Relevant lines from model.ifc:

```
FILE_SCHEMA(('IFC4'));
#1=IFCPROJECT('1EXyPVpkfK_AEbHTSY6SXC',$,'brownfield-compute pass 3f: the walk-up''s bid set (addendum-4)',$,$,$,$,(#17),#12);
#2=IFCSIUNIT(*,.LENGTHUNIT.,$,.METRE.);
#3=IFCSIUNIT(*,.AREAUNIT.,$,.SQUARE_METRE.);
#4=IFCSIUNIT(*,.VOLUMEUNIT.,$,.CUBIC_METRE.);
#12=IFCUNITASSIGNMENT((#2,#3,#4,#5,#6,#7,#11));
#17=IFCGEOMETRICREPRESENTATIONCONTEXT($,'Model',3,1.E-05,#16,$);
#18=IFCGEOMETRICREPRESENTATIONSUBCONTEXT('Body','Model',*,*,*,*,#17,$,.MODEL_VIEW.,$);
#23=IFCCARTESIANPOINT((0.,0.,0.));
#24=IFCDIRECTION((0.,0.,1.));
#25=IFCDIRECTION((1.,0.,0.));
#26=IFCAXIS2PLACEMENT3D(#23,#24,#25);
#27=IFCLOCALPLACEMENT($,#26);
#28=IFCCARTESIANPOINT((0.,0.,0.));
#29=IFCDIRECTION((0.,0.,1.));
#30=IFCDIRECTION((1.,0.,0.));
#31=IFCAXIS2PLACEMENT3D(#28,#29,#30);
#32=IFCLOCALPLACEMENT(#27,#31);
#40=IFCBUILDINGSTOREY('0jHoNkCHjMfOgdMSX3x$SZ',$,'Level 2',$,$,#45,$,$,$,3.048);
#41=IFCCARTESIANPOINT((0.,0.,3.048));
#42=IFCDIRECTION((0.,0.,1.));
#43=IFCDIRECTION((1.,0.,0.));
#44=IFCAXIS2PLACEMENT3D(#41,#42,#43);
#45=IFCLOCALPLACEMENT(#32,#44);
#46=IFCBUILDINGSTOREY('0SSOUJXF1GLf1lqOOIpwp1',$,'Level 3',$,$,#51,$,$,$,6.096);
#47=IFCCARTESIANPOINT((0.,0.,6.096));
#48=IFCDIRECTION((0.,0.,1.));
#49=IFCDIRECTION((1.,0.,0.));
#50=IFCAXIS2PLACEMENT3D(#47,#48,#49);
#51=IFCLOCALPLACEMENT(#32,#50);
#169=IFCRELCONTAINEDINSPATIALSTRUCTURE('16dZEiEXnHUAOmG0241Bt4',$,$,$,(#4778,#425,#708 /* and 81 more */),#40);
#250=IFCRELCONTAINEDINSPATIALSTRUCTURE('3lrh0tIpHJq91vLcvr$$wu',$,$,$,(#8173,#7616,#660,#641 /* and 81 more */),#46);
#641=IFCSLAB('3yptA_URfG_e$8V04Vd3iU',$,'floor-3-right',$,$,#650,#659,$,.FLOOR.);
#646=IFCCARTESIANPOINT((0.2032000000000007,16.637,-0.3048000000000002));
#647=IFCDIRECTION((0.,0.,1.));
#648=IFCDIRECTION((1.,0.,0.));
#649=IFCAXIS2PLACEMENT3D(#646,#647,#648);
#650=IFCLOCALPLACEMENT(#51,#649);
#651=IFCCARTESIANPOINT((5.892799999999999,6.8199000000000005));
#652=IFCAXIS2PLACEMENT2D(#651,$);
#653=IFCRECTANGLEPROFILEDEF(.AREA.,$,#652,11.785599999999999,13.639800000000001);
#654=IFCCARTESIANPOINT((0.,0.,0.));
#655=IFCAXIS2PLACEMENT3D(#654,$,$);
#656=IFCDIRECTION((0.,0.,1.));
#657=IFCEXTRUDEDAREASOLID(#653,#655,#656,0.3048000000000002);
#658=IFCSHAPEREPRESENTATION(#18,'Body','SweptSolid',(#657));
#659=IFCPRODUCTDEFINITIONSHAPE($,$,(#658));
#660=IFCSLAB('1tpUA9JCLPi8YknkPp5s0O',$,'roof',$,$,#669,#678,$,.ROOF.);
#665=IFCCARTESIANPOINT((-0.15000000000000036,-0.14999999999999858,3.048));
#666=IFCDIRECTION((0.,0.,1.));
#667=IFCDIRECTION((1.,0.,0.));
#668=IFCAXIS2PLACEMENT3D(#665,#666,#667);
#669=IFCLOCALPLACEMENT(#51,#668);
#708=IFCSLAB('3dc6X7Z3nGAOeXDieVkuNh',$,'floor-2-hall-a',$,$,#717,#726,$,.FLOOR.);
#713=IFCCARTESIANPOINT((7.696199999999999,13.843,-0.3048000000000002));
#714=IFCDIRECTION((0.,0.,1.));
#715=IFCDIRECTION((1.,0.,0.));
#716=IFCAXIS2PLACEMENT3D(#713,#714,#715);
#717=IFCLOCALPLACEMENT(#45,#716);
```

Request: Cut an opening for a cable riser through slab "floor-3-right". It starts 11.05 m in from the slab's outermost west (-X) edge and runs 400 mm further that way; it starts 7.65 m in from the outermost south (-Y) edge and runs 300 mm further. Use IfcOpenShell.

```python
import numpy as np
import ifcopenshell
import ifcopenshell.api.feature
import ifcopenshell.api.geometry
import ifcopenshell.api.root
import ifcopenshell.geom
import ifcopenshell.util.placement
import ifcopenshell.util.representation
import ifcopenshell.util.shape
import ifcopenshell.util.unit

model = ifcopenshell.open("model.ifc")
unit_scale = ifcopenshell.util.unit.calculate_unit_scale(model)
settings = ifcopenshell.geom.settings()


def volume(element):
    """Net volume in cubic metres, openings subtracted."""
    shape = ifcopenshell.geom.create_shape(settings, element)
    return ifcopenshell.util.shape.get_volume(shape.geometry)


slab = model.by_guid("3yptA_URfG_e$8V04Vd3iU")
before = volume(slab)

# Extent in the slab's own axes, in metres. The edges named are its -X and -Y sides.
slab_shape = ifcopenshell.geom.create_shape(settings, slab)
vertices = ifcopenshell.util.shape.get_vertices(slab_shape.geometry)
x_min, y_min, bottom = vertices.min(axis=0)
top = vertices[:, 2].max()

opening = ifcopenshell.api.root.create_entity(model, ifc_class="IfcOpeningElement", name="Cable riser opening", predefined_type="OPENING")
context = ifcopenshell.util.representation.get_context(model, "Model", "Body", "MODEL_VIEW")
width, depth = 0.4, 0.3
outline = [(0.0, 0.0), (width, 0.0), (width, depth), (0.0, depth), (0.0, 0.0)]
# Overshoot both faces by 50 mm so the cut is clean.
shape = ifcopenshell.api.geometry.add_slab_representation(
    model, context=context, depth=top - bottom + 0.1, polyline=outline
)
ifcopenshell.api.geometry.assign_representation(model, product=opening, representation=shape)

matrix = ifcopenshell.util.placement.get_local_placement(slab.ObjectPlacement)
matrix[:, 3] = matrix @ np.append(np.array([x_min + 11.05, y_min + 7.65, bottom - 0.05]) / unit_scale, 1.0)
ifcopenshell.api.geometry.edit_object_placement(model, product=opening, matrix=matrix, is_si=False)
ifcopenshell.api.feature.add_feature(model, feature=opening, element=slab)

after = volume(slab)

print(f"slab volume {before:.3f} -> {after:.3f} m3")

model.write("model_updated.ifc")
```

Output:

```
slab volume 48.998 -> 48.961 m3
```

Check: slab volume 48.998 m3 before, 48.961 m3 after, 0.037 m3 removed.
